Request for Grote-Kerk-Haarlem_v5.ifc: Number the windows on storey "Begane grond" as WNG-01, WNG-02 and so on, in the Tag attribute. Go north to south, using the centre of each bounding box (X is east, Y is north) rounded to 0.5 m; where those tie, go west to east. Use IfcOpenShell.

First a look at what the model holds.

```python
import ifcopenshell
import ifcopenshell.util.element
import ifcopenshell.util.placement

model = ifcopenshell.open("Grote-Kerk-Haarlem_v5.ifc")
print(model.schema)
storey = next(s for s in model.by_type("IfcBuildingStorey") if s.Name == "Begane grond")
windows = [e for e in ifcopenshell.util.element.get_decomposition(storey) if e.is_a("IfcWindow")]
for e in sorted(windows, key=lambda e: e.id()):
    origin = ifcopenshell.util.placement.get_local_placement(e.ObjectPlacement)[:3, 3]
    print(e.id(), e.Tag, e.Name, origin.round(2) + 0.0, sep=" | ")
```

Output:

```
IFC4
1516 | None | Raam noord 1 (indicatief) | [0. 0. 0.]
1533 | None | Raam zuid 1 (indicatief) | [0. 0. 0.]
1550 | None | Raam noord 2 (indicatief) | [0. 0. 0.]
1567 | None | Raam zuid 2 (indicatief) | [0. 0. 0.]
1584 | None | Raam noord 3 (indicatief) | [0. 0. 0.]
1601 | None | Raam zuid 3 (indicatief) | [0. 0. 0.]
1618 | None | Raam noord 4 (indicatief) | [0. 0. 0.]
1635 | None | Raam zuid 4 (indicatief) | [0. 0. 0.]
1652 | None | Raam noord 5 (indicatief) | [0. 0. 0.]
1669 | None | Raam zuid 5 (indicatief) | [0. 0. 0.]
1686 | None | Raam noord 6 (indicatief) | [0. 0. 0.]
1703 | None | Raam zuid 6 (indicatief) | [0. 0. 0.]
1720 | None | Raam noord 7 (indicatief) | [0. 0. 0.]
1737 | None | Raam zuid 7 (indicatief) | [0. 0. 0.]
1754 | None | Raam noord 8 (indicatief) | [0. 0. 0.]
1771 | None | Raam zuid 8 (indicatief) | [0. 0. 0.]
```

```python
import ifcopenshell
import ifcopenshell.geom
import ifcopenshell.util.element
import ifcopenshell.util.shape

model = ifcopenshell.open("Grote-Kerk-Haarlem_v5.ifc")
settings = ifcopenshell.geom.settings()
settings.set("use-world-coords", True)


def centre(element):
    shape = ifcopenshell.geom.create_shape(settings, element)
    return ifcopenshell.util.shape.get_bbox_centroid(shape.geometry)


storey = next(s for s in model.by_type("IfcBuildingStorey") if s.Name == "Begane grond")
windows = [e for e in ifcopenshell.util.element.get_decomposition(storey) if e.is_a("IfcWindow")]

# Insertion points can sit at a corner or the storey origin, so sort by the geometry (in metres).
centres = {e: centre(e) for e in windows}
windows.sort(key=lambda e: (-round(centres[e][1] / 0.5), centres[e][0]))

for i, e in enumerate(windows, start=1):
    number = f"WNG-{i:02d}"
    e.Tag = number
    print(e.id(), number)

model.write("Grote-Kerk-Haarlem_v5-out.ifc")
```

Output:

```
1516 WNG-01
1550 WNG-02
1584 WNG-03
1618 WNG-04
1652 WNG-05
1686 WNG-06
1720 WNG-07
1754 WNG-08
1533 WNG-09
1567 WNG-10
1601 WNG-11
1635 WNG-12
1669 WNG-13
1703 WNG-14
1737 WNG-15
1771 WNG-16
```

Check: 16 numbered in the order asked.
